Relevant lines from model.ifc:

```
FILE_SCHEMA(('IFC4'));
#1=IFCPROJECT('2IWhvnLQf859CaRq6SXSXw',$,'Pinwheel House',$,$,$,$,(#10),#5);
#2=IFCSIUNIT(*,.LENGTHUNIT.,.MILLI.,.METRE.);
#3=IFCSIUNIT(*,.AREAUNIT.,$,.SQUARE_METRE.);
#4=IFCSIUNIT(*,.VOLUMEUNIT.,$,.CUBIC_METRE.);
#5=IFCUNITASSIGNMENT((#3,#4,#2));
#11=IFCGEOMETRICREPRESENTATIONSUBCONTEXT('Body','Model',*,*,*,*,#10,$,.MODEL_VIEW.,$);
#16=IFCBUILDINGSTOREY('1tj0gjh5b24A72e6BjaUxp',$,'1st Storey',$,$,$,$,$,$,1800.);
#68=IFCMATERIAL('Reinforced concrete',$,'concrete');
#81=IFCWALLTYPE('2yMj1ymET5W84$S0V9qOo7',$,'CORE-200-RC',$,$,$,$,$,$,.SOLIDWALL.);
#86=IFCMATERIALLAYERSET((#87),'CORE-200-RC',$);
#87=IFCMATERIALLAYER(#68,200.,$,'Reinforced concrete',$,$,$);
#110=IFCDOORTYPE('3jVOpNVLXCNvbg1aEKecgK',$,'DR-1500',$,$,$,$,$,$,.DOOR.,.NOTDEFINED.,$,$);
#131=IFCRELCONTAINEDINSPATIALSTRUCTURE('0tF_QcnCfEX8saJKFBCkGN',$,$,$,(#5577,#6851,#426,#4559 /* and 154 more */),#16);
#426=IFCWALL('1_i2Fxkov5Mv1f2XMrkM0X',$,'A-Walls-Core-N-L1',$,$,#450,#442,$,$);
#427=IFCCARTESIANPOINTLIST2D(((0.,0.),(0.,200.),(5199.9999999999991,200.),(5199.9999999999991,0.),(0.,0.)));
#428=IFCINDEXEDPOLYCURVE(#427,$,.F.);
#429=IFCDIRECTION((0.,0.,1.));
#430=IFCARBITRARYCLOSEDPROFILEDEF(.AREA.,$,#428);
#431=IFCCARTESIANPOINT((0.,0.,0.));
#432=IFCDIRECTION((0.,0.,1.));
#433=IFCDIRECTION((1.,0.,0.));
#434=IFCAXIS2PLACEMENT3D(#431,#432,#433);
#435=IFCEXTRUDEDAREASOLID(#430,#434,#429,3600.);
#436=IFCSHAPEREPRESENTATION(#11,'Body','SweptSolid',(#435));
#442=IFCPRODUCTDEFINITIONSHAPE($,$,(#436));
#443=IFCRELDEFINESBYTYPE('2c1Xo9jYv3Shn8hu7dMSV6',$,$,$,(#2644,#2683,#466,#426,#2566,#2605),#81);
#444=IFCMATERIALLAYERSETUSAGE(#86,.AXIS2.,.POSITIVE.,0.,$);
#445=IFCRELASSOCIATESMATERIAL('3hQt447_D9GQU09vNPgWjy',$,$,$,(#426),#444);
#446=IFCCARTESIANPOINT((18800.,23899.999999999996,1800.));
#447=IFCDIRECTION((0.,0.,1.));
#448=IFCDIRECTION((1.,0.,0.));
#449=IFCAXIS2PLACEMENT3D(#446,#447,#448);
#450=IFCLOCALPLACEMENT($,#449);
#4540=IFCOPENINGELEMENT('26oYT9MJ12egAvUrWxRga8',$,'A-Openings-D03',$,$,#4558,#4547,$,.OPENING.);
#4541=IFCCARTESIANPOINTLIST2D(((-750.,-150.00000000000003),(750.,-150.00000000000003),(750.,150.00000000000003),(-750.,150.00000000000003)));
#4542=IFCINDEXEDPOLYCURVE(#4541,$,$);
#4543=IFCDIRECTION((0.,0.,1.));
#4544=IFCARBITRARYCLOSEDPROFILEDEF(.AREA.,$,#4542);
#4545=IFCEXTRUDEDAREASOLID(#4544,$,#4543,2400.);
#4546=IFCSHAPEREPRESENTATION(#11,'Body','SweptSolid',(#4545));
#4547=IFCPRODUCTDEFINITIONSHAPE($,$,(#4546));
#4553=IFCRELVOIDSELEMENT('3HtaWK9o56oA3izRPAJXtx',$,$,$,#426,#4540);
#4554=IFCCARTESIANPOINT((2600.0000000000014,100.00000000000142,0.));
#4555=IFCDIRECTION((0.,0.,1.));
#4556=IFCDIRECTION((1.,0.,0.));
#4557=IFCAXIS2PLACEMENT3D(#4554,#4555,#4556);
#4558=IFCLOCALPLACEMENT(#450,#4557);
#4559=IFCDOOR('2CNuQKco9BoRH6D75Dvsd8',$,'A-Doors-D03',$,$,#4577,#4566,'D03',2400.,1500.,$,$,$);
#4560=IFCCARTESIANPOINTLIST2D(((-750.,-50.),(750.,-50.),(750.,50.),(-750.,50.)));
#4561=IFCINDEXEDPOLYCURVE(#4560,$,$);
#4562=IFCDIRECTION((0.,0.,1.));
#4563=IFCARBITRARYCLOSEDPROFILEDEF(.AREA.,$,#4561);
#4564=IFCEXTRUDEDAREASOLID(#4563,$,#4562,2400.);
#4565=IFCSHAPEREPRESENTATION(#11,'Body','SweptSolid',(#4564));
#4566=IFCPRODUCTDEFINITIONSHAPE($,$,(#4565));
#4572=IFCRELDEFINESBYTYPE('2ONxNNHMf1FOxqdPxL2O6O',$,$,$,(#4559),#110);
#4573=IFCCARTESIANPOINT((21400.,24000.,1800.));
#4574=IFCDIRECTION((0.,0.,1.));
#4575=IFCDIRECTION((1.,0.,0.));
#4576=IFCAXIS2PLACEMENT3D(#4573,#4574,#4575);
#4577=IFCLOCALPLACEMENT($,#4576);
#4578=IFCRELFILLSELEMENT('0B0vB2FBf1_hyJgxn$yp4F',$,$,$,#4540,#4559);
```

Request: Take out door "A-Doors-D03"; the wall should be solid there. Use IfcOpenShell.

```python
import ifcopenshell
import ifcopenshell.api.feature
import ifcopenshell.api.root
import ifcopenshell.geom
import ifcopenshell.util.shape

model = ifcopenshell.open("model.ifc")
settings = ifcopenshell.geom.settings()


def volume(element):
    """Net volume in cubic metres, openings subtracted."""
    shape = ifcopenshell.geom.create_shape(settings, element)
    return ifcopenshell.util.shape.get_volume(shape.geometry)


door = model.by_guid("2CNuQKco9BoRH6D75Dvsd8")
opening = door.FillsVoids[0].RelatingOpeningElement
wall = opening.VoidsElements[0].RelatingBuildingElement
before = volume(wall)

ifcopenshell.api.root.remove_product(model, product=door)
ifcopenshell.api.feature.remove_feature(model, feature=opening)

after = volume(wall)

print(f"wall volume {before:.3f} -> {after:.3f} m3")

model.write("model_edited.ifc")
```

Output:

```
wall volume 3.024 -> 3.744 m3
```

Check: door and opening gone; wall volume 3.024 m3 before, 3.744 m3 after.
